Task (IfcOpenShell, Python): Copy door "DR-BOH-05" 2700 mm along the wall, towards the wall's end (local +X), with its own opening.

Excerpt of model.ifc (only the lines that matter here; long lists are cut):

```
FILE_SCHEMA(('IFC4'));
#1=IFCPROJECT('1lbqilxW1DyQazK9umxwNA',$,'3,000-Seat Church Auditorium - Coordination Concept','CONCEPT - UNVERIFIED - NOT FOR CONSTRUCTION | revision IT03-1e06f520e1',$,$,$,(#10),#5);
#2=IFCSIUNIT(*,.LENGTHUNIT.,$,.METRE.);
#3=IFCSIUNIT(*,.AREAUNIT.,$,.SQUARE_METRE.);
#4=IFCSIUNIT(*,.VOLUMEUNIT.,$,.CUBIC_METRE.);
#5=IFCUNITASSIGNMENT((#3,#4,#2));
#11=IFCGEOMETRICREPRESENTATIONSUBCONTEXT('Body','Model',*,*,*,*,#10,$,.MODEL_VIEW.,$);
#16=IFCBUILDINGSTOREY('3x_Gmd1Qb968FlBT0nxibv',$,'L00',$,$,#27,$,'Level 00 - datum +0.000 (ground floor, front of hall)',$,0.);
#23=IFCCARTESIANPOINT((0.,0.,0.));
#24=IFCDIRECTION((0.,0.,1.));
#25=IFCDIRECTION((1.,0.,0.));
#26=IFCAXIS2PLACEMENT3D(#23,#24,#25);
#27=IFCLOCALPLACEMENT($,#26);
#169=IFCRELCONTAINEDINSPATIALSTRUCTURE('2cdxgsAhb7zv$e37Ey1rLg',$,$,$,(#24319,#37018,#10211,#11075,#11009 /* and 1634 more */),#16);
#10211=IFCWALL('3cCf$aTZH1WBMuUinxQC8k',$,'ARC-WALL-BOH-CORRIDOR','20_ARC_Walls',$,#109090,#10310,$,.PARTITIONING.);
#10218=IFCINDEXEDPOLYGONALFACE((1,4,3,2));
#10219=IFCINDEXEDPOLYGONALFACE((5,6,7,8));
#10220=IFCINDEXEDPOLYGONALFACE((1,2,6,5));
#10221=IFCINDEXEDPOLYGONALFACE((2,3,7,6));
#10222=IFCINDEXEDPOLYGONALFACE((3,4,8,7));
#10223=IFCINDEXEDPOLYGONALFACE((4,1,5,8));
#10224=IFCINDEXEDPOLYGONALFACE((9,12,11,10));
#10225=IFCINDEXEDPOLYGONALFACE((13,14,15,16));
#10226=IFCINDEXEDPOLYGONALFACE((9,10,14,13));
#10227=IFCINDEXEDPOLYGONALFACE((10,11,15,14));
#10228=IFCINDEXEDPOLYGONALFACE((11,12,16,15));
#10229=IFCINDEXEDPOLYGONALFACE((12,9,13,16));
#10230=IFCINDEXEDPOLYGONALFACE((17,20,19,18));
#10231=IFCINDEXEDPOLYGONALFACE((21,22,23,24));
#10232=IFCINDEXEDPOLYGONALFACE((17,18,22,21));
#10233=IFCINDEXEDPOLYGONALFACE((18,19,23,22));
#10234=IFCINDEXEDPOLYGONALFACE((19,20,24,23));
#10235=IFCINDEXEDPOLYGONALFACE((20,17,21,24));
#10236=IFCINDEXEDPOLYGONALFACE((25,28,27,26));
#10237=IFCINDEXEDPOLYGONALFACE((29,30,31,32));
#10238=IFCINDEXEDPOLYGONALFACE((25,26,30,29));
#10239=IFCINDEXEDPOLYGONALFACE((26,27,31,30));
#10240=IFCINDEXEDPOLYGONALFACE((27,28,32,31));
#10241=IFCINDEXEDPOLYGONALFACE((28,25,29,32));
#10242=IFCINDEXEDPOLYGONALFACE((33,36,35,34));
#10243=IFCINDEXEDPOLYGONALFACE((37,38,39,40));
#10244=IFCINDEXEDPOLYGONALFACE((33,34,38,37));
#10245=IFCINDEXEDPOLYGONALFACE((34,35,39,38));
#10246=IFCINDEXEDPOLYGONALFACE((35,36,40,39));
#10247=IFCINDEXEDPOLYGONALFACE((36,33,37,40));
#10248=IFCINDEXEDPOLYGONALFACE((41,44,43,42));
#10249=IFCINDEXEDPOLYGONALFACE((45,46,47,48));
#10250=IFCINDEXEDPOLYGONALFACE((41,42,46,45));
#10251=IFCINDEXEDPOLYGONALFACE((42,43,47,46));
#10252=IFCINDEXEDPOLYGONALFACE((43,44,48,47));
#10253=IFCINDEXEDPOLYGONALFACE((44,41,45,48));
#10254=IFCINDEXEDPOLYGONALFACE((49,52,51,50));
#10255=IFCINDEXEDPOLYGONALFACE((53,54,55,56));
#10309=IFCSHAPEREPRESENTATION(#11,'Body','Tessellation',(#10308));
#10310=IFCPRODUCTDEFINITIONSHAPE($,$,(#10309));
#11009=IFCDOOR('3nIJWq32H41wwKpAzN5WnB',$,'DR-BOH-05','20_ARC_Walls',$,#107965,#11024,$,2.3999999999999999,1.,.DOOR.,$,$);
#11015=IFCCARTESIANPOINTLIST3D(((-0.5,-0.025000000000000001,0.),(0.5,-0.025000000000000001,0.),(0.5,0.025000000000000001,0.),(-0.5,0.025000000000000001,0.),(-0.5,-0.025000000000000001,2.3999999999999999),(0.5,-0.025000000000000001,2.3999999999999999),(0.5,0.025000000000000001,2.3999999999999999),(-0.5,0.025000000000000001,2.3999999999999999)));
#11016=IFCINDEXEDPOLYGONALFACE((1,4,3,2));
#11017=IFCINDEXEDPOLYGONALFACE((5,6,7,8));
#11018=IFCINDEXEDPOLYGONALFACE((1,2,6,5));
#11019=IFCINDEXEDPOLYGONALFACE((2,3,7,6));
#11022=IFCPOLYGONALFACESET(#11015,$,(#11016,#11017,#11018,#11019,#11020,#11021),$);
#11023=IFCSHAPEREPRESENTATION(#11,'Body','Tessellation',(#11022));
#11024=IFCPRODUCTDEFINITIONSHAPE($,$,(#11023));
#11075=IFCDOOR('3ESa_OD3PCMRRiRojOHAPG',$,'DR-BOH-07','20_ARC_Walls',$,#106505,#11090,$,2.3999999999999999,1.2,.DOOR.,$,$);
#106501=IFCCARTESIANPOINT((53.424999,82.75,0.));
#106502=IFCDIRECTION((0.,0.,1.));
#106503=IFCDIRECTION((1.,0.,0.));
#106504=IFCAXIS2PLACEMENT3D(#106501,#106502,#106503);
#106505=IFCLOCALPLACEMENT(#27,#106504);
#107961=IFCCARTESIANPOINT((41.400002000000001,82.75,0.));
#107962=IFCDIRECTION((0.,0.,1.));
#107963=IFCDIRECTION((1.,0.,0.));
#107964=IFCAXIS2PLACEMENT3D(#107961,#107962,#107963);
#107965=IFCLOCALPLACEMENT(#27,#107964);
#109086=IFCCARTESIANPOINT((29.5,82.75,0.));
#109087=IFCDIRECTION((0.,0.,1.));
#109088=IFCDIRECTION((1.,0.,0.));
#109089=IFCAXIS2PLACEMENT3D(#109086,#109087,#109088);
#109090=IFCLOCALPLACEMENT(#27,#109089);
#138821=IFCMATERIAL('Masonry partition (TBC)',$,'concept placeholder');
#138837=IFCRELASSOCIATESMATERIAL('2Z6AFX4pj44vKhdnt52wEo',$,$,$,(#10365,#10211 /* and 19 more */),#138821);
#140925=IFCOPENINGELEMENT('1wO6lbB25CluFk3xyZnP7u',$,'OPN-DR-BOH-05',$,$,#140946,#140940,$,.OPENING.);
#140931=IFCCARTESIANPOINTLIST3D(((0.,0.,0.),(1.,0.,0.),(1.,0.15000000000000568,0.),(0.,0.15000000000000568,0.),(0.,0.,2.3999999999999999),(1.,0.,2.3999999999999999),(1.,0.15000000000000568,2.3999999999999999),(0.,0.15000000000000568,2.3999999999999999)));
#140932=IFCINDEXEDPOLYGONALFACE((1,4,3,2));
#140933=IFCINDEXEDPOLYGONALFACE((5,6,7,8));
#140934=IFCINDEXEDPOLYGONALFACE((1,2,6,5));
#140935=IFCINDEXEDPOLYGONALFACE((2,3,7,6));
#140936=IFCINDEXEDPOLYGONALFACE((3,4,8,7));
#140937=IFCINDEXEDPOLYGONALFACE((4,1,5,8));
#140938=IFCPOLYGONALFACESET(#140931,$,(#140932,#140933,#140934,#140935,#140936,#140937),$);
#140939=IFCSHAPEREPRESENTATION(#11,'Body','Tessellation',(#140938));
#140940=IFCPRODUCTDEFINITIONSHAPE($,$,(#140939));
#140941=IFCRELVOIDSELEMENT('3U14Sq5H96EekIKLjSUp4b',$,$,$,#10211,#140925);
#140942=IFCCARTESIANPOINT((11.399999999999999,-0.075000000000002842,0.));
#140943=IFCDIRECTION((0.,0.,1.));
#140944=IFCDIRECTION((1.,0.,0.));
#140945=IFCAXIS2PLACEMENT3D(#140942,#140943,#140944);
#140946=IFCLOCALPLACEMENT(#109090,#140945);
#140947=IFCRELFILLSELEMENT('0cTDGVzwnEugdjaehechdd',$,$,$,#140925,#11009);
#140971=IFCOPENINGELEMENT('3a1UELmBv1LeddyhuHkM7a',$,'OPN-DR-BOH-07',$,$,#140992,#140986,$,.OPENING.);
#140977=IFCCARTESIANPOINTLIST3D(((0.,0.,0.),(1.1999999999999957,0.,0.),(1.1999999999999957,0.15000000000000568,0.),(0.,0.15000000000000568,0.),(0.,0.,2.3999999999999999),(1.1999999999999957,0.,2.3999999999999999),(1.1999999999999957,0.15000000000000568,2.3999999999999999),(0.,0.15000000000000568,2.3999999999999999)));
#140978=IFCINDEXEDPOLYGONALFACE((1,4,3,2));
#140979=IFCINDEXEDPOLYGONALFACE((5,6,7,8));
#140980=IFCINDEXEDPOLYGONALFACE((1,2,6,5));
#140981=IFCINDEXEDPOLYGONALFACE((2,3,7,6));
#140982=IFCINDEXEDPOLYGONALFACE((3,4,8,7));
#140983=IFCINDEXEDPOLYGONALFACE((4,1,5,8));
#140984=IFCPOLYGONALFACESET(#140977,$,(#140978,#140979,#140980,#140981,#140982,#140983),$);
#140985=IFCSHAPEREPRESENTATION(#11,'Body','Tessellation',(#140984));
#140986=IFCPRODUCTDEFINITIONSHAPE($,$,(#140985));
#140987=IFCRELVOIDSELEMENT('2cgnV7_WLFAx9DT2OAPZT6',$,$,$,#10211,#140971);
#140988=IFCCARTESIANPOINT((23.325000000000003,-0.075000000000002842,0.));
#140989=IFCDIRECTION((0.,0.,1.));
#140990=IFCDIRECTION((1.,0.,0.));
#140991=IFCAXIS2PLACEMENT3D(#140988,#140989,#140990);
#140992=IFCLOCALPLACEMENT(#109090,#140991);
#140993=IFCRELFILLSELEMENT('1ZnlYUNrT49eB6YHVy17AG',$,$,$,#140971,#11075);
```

```python
import ifcopenshell
import ifcopenshell.api.feature
import ifcopenshell.api.geometry
import ifcopenshell.api.root
import ifcopenshell.geom
import ifcopenshell.util.element
import ifcopenshell.util.placement
import ifcopenshell.util.shape

model = ifcopenshell.open("model.ifc")
settings = ifcopenshell.geom.settings()


def volume(element):
    """Net volume in cubic metres, openings subtracted."""
    shape = ifcopenshell.geom.create_shape(settings, element)
    return ifcopenshell.util.shape.get_volume(shape.geometry)


door = model.by_id(11009)
opening = door.FillsVoids[0].RelatingOpeningElement
wall = opening.VoidsElements[0].RelatingBuildingElement
before = volume(wall)
shift = ifcopenshell.util.placement.get_local_placement(wall.ObjectPlacement)[:3, 0] * 2.7

# copy_class copies the void relationship, type, container and properties, but no geometry.
new_opening = ifcopenshell.api.root.copy_class(model, product=opening)
new_opening.Representation = ifcopenshell.util.element.copy_deep(
    model, opening.Representation, exclude=["IfcGeometricRepresentationContext", "IfcRepresentationMap"]
)
new_door = ifcopenshell.api.root.copy_class(model, product=door)
new_door.Representation = ifcopenshell.util.element.copy_deep(
    model, door.Representation, exclude=["IfcGeometricRepresentationContext", "IfcRepresentationMap"]
)
ifcopenshell.api.feature.add_filling(model, opening=new_opening, element=new_door)

for old, new in ((opening, new_opening), (door, new_door)):
    matrix = ifcopenshell.util.placement.get_local_placement(old.ObjectPlacement)
    matrix[:3, 3] += shift
    ifcopenshell.api.geometry.edit_object_placement(model, product=new, matrix=matrix, is_si=False)

after = volume(wall)

print(f"wall volume {before:.3f} -> {after:.3f} m3")

model.write("model_edited.ifc")
```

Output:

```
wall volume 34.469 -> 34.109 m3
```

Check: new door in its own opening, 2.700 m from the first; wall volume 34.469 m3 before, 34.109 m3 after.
